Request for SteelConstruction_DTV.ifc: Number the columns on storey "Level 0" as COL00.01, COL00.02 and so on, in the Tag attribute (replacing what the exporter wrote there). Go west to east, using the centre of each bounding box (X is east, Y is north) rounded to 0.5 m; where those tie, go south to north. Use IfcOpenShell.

First a look at what the model holds.

```python
import ifcopenshell
import ifcopenshell.util.element
import ifcopenshell.util.placement

model = ifcopenshell.open("SteelConstruction_DTV.ifc")
print(model.schema)
storey = next(s for s in model.by_type("IfcBuildingStorey") if s.Name == "Level 0")
columns = [e for e in ifcopenshell.util.element.get_decomposition(storey) if e.is_a("IfcColumn")]
for e in sorted(columns, key=lambda e: e.id()):
    origin = ifcopenshell.util.placement.get_local_placement(e.ObjectPlacement)[:3, 3]
    print(e.id(), e.Tag, e.Name, origin.round(2) + 0.0, sep=" | ")
```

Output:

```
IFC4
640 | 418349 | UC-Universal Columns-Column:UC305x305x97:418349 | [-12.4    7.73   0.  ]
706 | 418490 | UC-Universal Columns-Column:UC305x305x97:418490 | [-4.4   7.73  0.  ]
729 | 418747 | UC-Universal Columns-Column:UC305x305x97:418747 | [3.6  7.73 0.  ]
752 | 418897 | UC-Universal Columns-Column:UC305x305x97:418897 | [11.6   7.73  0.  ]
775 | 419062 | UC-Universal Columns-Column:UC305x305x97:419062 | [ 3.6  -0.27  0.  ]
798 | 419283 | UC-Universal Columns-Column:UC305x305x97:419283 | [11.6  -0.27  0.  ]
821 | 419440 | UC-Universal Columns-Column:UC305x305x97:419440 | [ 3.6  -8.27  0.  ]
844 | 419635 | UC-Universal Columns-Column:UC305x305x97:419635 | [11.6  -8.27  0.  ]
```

```python
import ifcopenshell
import ifcopenshell.geom
import ifcopenshell.util.element
import ifcopenshell.util.shape

model = ifcopenshell.open("SteelConstruction_DTV.ifc")
settings = ifcopenshell.geom.settings()
settings.set("use-world-coords", True)


def centre(element):
    shape = ifcopenshell.geom.create_shape(settings, element)
    return ifcopenshell.util.shape.get_bbox_centroid(shape.geometry)


storey = next(s for s in model.by_type("IfcBuildingStorey") if s.Name == "Level 0")
columns = [e for e in ifcopenshell.util.element.get_decomposition(storey) if e.is_a("IfcColumn")]

# Insertion points can sit at a corner or the storey origin, so sort by the geometry (in metres).
centres = {e: centre(e) for e in columns}
columns.sort(key=lambda e: (round(centres[e][0] / 0.5), centres[e][1]))

for i, e in enumerate(columns, start=1):
    number = f"COL00.{i:02d}"
    e.Tag = number
    print(e.id(), number)

model.write("SteelConstruction_DTV_updated.ifc")
```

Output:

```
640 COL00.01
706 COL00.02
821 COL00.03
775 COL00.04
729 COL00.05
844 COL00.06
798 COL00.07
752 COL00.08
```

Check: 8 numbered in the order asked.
